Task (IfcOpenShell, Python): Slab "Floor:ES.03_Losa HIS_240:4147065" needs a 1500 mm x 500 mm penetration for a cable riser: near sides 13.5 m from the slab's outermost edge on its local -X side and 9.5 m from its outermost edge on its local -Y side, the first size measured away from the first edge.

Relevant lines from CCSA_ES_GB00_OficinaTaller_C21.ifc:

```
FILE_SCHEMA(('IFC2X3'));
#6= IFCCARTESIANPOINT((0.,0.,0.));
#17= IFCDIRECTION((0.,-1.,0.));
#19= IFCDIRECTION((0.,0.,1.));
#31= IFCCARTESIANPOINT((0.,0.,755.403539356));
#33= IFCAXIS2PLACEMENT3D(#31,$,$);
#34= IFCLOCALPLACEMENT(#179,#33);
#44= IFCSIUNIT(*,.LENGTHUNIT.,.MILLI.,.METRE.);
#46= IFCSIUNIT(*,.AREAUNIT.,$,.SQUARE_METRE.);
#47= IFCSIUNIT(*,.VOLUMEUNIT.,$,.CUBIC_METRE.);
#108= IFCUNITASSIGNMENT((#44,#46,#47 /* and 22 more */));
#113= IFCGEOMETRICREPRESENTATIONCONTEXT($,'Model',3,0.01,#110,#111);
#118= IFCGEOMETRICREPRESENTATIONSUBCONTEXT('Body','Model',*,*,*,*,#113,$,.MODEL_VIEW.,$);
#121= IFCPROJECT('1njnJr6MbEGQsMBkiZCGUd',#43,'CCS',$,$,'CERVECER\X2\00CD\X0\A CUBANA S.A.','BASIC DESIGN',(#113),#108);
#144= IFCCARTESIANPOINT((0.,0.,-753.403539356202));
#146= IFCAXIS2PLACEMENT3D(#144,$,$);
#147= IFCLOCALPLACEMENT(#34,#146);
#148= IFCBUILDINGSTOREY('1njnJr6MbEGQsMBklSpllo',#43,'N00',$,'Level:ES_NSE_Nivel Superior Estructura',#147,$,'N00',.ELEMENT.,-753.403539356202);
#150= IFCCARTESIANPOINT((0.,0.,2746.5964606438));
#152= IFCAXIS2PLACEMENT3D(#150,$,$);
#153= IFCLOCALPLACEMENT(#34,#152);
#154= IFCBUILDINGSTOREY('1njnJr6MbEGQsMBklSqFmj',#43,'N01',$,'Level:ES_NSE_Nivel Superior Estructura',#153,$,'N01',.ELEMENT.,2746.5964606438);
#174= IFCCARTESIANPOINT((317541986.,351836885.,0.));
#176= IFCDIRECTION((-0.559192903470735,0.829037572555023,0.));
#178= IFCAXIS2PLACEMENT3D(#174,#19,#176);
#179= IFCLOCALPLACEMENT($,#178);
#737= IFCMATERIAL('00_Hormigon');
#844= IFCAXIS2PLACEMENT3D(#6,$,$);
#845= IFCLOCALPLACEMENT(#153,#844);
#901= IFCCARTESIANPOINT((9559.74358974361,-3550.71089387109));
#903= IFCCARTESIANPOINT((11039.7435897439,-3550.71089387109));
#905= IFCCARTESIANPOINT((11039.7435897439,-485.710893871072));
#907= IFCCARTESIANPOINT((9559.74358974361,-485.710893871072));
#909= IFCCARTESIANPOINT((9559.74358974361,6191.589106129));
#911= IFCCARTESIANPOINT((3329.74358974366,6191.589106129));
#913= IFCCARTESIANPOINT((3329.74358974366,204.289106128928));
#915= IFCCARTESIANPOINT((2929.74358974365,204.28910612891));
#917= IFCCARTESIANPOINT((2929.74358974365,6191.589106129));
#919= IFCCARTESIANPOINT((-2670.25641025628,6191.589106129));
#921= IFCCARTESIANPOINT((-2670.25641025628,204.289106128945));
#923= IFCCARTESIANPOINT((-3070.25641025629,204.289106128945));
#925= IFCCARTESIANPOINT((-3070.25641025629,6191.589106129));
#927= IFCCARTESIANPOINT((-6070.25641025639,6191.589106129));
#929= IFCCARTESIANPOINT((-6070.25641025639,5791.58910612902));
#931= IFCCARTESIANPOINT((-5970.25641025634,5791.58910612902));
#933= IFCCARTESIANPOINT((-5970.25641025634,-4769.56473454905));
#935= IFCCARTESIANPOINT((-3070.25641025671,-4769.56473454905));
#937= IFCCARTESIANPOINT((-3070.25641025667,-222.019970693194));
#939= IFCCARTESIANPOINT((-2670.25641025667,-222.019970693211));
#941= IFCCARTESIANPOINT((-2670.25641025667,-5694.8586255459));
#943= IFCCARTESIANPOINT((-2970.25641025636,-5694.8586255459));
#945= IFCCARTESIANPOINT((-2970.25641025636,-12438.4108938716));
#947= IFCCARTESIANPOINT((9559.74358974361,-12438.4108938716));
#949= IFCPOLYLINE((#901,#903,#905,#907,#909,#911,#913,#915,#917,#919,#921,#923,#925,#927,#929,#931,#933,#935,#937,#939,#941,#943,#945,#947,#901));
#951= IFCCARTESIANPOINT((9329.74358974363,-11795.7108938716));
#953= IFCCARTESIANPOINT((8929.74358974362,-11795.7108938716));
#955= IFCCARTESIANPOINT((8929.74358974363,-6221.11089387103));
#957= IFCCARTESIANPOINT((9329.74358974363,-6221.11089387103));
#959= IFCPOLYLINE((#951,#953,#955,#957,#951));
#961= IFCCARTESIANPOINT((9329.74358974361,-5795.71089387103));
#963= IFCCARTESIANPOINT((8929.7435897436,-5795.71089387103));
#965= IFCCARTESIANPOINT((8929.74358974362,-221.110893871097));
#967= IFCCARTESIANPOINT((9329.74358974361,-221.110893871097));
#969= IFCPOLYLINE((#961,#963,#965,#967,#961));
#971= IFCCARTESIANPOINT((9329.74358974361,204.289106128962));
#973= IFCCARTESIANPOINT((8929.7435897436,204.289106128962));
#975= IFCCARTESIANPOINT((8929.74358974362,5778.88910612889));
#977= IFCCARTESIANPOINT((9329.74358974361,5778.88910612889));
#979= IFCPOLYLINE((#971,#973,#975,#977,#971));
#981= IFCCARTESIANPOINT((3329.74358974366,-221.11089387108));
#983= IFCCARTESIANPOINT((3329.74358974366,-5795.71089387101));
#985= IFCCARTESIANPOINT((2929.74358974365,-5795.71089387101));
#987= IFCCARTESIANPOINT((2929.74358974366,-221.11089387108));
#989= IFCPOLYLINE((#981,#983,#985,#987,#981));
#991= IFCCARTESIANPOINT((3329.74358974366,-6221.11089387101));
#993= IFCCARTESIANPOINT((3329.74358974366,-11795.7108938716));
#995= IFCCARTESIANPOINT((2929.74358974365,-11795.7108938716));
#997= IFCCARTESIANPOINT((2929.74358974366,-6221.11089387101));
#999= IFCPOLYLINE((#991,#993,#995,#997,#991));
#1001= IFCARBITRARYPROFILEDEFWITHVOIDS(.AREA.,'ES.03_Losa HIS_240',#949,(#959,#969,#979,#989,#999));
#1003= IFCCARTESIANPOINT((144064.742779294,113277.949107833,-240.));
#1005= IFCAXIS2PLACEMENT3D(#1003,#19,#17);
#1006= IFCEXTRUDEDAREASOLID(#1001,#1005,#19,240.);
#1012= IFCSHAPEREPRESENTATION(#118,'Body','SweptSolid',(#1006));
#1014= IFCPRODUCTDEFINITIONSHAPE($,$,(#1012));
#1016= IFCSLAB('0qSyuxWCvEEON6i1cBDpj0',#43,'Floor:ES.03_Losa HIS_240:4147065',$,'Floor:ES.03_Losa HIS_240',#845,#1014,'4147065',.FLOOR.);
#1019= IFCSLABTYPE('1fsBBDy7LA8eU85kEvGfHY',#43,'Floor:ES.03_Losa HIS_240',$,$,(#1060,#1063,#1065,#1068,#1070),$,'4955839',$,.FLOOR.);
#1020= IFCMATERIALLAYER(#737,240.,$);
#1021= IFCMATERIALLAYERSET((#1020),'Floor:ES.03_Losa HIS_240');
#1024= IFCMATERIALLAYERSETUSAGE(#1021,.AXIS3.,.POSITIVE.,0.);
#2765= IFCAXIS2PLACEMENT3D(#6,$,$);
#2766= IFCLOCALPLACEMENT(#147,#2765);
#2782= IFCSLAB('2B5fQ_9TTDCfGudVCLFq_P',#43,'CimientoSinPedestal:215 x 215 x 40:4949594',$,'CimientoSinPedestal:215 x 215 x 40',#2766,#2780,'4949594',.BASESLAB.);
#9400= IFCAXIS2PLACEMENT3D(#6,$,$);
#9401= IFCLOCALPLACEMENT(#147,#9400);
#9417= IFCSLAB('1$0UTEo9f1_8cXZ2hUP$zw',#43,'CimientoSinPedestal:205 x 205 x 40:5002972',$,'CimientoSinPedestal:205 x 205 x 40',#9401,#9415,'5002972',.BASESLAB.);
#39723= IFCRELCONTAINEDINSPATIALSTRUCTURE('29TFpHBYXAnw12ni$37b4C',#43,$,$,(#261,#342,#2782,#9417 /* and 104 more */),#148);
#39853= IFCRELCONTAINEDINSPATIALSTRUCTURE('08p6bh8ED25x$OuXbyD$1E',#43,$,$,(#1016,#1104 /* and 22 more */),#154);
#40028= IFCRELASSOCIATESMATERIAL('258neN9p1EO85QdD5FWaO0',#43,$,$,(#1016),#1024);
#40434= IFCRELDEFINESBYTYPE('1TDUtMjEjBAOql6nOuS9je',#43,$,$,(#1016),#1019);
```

```python
import numpy as np
import ifcopenshell
import ifcopenshell.api.feature
import ifcopenshell.api.geometry
import ifcopenshell.api.root
import ifcopenshell.geom
import ifcopenshell.util.placement
import ifcopenshell.util.representation
import ifcopenshell.util.shape
import ifcopenshell.util.unit

model = ifcopenshell.open("CCSA_ES_GB00_OficinaTaller_C21.ifc")
unit_scale = ifcopenshell.util.unit.calculate_unit_scale(model)
settings = ifcopenshell.geom.settings()


def volume(element):
    """Net volume in cubic metres, openings subtracted."""
    shape = ifcopenshell.geom.create_shape(settings, element)
    return ifcopenshell.util.shape.get_volume(shape.geometry)


slab = model.by_guid("0qSyuxWCvEEON6i1cBDpj0")
before = volume(slab)

# Extent in the slab's own axes, in metres. The edges named are its -X and -Y sides.
slab_shape = ifcopenshell.geom.create_shape(settings, slab)
vertices = ifcopenshell.util.shape.get_vertices(slab_shape.geometry)
x_min, y_min, bottom = vertices.min(axis=0)
top = vertices[:, 2].max()

opening = ifcopenshell.api.root.create_entity(model, ifc_class="IfcOpeningElement", name="Cable riser opening")
context = ifcopenshell.util.representation.get_context(model, "Model", "Body", "MODEL_VIEW")
width, depth = 1.5, 0.5
outline = [(0.0, 0.0), (width, 0.0), (width, depth), (0.0, depth), (0.0, 0.0)]
# Overshoot both faces by 50 mm so the cut is clean.
shape = ifcopenshell.api.geometry.add_slab_representation(
    model, context=context, depth=top - bottom + 0.1, polyline=outline
)
ifcopenshell.api.geometry.assign_representation(model, product=opening, representation=shape)

matrix = ifcopenshell.util.placement.get_local_placement(slab.ObjectPlacement)
matrix[:, 3] = matrix @ np.append(np.array([x_min + 13.5, y_min + 9.5, bottom - 0.05]) / unit_scale, 1.0)
ifcopenshell.api.geometry.edit_object_placement(model, product=opening, matrix=matrix, is_si=False)
ifcopenshell.api.feature.add_feature(model, feature=opening, element=slab)

after = volume(slab)

print(f"slab volume {before:.3f} -> {after:.3f} m3")

model.write("CCSA_ES_GB00_OficinaTaller_C21_rev.ifc")
```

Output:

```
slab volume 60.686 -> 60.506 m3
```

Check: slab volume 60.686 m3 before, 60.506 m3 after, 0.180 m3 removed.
